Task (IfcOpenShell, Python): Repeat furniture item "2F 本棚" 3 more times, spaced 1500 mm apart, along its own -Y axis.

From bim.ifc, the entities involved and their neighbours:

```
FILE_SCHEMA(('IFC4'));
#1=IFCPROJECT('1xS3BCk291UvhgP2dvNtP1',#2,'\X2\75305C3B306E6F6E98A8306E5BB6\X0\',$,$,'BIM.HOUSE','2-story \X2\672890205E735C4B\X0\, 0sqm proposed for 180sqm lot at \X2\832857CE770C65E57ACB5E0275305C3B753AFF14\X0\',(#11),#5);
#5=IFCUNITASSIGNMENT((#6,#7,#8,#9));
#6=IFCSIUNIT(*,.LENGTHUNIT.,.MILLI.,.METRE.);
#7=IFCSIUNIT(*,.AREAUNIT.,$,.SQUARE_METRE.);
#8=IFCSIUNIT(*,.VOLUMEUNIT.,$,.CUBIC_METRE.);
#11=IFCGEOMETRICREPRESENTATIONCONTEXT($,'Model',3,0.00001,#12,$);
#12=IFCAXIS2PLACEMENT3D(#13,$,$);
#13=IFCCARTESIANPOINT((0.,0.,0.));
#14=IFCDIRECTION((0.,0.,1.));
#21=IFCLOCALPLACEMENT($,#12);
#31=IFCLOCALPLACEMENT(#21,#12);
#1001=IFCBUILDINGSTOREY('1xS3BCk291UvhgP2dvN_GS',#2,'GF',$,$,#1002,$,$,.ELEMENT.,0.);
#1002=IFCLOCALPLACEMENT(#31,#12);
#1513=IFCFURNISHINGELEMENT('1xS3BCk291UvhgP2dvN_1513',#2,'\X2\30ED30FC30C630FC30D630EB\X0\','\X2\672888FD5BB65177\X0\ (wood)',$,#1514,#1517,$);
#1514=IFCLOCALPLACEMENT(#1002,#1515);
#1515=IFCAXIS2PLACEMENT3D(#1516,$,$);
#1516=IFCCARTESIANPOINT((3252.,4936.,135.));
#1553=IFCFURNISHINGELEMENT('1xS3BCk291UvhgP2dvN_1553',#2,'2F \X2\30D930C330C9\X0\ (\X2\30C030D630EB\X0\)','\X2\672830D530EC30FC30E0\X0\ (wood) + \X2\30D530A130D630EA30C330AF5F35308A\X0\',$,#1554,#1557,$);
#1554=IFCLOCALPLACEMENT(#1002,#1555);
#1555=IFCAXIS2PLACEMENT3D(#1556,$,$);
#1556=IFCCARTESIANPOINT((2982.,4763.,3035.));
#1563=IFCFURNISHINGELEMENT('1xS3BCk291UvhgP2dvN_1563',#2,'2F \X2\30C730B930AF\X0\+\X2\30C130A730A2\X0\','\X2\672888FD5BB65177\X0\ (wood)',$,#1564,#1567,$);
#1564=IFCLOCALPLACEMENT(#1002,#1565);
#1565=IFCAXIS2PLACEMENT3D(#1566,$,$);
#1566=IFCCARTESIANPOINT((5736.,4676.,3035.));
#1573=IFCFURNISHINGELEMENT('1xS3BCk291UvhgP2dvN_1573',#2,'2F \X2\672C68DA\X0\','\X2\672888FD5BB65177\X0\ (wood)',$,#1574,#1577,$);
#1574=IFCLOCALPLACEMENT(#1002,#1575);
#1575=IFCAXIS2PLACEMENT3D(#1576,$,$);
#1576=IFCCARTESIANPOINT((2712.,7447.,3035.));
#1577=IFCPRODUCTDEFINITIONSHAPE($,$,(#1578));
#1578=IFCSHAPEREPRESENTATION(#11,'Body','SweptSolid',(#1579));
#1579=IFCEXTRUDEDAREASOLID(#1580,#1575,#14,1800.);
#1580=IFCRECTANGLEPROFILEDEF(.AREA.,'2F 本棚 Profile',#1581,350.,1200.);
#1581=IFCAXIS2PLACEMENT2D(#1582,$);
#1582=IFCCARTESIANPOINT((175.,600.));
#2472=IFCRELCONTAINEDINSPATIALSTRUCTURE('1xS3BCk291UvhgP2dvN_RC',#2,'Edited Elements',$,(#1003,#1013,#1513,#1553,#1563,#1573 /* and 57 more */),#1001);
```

```python
import ifcopenshell
import ifcopenshell.api.geometry
import ifcopenshell.api.root
import ifcopenshell.util.element
import ifcopenshell.util.placement

model = ifcopenshell.open("bim.ifc")


def reuse_history(source, copy):
    """copy_class also copies each property set's owner history, people and application; keep the originals."""
    for rel in copy.IsDefinedBy:
        if rel.is_a("IfcRelDefinesByProperties") and (history := rel.RelatingPropertyDefinition.OwnerHistory):
            rel.RelatingPropertyDefinition.OwnerHistory = source.OwnerHistory
            ifcopenshell.util.element.remove_deep2(model, history)


source = model.by_id(1573)
base = ifcopenshell.util.placement.get_local_placement(source.ObjectPlacement)
step = -base[:3, 1] * 1500.0

for i in range(1, 4):
    copy = ifcopenshell.api.root.copy_class(model, product=source)
    copy.Representation = ifcopenshell.util.element.copy_deep(
        model, source.Representation, exclude=["IfcGeometricRepresentationContext", "IfcRepresentationMap"]
    )
    reuse_history(source, copy)
    matrix = base.copy()
    matrix[:3, 3] += i * step
    print("added at", matrix[:3, 3].round(3) + 0.0)
    ifcopenshell.api.geometry.edit_object_placement(model, product=copy, matrix=matrix, is_si=False)

model.write("bim_rev.ifc")
```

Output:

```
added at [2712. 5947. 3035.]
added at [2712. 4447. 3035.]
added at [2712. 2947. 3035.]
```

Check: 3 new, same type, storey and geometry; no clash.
